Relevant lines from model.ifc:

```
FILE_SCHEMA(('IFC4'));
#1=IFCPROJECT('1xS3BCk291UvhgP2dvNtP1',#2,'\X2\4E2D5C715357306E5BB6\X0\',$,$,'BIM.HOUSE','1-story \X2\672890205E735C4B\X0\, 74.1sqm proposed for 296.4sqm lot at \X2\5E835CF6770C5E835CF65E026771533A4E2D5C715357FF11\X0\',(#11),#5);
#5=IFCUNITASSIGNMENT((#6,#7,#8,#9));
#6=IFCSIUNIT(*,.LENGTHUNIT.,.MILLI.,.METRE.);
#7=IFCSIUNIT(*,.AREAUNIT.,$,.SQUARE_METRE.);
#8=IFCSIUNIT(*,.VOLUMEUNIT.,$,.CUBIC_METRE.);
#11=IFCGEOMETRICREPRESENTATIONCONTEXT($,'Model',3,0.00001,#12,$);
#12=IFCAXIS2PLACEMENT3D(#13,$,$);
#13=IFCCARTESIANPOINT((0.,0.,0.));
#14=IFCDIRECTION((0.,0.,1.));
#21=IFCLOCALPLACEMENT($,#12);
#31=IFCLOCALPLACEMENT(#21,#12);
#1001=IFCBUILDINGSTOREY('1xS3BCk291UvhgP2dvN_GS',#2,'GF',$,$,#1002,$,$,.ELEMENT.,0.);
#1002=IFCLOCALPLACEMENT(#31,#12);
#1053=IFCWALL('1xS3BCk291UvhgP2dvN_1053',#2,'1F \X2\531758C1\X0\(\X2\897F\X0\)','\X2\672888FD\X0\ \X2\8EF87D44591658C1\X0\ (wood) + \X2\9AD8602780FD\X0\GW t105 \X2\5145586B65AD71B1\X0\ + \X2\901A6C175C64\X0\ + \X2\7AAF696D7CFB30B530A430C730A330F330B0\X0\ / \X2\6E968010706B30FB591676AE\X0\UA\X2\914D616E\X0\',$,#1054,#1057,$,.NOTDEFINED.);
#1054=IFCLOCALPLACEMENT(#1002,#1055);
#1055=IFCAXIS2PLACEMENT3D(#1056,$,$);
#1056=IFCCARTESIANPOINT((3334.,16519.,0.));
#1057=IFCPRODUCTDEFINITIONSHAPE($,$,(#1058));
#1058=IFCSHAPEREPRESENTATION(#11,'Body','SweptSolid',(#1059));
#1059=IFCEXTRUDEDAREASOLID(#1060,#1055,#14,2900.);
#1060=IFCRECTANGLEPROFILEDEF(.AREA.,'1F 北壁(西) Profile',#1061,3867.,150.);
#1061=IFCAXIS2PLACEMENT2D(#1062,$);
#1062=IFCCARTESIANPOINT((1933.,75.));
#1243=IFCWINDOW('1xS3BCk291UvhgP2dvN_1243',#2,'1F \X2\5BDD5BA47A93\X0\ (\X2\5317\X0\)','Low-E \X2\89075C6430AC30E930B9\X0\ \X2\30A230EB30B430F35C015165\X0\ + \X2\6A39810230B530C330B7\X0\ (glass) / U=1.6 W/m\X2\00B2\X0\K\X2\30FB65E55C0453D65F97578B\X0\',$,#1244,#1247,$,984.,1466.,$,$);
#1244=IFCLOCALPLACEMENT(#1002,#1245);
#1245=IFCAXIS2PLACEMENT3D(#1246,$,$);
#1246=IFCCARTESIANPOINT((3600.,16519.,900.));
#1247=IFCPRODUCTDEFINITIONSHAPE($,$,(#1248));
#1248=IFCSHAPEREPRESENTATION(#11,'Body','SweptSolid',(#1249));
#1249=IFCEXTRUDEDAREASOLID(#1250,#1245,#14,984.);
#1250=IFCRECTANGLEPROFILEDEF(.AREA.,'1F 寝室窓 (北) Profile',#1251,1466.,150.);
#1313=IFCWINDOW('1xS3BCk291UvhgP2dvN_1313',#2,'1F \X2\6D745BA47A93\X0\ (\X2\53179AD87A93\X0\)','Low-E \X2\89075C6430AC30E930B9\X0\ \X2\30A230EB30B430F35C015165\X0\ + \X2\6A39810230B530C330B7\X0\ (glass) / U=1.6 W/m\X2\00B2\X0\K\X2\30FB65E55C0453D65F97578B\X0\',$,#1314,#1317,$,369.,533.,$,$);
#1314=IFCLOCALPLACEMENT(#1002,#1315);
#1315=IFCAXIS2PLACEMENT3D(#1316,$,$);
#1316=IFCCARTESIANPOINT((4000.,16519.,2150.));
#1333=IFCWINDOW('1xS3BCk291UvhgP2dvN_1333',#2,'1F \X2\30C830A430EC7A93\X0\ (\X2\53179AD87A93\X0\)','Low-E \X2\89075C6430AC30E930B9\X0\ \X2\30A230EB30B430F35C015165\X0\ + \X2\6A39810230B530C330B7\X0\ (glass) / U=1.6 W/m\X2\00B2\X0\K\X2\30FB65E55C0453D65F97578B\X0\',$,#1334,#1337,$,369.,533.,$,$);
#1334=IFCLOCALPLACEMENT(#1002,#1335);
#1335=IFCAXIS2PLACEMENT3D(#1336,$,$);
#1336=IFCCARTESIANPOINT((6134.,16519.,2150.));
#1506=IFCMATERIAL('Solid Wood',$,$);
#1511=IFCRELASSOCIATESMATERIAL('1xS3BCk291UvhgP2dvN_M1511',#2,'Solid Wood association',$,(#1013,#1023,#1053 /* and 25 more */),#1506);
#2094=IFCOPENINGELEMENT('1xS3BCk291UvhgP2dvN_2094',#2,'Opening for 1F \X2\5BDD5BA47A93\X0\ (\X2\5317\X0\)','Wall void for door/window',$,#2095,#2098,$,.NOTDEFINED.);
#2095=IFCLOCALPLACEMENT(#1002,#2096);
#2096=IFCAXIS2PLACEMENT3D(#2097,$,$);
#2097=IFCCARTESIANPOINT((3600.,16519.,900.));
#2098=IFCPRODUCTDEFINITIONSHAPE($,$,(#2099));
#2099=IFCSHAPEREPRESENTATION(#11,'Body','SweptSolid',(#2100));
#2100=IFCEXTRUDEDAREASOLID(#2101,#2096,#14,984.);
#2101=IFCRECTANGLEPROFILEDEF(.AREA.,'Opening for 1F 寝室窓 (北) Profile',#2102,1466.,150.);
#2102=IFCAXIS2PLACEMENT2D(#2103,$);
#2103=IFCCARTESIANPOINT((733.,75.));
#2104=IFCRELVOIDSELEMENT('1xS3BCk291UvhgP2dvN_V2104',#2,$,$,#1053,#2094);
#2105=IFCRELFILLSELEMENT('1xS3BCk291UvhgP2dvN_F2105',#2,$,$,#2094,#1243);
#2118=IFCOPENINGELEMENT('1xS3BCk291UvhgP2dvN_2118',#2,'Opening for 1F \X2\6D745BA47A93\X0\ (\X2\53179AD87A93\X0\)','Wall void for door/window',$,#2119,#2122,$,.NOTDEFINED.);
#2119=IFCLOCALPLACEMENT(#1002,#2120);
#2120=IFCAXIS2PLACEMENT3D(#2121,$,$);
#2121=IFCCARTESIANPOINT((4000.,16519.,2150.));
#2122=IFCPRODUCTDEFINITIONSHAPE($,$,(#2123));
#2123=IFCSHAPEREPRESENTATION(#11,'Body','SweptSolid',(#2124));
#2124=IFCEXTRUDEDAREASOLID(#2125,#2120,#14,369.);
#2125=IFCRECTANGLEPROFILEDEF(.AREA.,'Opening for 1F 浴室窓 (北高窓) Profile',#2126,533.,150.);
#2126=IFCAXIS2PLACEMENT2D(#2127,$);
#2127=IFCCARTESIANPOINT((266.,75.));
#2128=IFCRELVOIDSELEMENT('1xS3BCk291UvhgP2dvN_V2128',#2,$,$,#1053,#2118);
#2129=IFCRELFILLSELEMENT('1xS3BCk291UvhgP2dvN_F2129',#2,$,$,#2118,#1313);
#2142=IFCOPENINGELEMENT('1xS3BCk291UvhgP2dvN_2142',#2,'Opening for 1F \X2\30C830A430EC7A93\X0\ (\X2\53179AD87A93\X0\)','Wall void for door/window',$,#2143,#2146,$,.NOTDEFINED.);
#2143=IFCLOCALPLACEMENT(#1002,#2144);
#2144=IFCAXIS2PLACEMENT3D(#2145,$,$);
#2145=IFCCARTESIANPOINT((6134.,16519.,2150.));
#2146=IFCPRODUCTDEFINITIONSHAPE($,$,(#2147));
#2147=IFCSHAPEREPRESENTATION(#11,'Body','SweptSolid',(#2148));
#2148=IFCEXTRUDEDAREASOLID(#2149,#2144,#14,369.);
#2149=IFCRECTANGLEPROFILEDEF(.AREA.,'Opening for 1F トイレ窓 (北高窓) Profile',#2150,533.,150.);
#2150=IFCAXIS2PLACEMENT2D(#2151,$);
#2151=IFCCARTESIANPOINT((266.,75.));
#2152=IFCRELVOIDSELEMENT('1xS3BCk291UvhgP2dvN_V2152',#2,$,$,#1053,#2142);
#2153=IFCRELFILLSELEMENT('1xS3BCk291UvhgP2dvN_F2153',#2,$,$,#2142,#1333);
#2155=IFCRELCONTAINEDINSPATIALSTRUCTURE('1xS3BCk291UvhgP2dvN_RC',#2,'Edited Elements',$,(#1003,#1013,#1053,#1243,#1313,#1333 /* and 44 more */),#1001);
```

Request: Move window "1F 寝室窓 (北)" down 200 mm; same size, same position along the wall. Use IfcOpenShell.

```python
import numpy as np
import ifcopenshell
import ifcopenshell.api.geometry
import ifcopenshell.util.placement
import ifcopenshell.util.unit

model = ifcopenshell.open("model.ifc")
unit_scale = ifcopenshell.util.unit.calculate_unit_scale(model)

window = model.by_guid("1xS3BCk291UvhgP2dvN_1243")
opening = window.FillsVoids[0].RelatingOpeningElement
dz = -200.0

shift = np.array([0.0, 0.0, dz])
# The window is not placed relative to its opening, so move both.
for product in (opening, window):
    matrix = ifcopenshell.util.placement.get_local_placement(product.ObjectPlacement)
    matrix[:3, 3] += shift
    ifcopenshell.api.geometry.edit_object_placement(model, product=product, matrix=matrix, is_si=False)

print(f"moved by {dz * unit_scale:+.3f} m")

model.write("model_v2.ifc")
```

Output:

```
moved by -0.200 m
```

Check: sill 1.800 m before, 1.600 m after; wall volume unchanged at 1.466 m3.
